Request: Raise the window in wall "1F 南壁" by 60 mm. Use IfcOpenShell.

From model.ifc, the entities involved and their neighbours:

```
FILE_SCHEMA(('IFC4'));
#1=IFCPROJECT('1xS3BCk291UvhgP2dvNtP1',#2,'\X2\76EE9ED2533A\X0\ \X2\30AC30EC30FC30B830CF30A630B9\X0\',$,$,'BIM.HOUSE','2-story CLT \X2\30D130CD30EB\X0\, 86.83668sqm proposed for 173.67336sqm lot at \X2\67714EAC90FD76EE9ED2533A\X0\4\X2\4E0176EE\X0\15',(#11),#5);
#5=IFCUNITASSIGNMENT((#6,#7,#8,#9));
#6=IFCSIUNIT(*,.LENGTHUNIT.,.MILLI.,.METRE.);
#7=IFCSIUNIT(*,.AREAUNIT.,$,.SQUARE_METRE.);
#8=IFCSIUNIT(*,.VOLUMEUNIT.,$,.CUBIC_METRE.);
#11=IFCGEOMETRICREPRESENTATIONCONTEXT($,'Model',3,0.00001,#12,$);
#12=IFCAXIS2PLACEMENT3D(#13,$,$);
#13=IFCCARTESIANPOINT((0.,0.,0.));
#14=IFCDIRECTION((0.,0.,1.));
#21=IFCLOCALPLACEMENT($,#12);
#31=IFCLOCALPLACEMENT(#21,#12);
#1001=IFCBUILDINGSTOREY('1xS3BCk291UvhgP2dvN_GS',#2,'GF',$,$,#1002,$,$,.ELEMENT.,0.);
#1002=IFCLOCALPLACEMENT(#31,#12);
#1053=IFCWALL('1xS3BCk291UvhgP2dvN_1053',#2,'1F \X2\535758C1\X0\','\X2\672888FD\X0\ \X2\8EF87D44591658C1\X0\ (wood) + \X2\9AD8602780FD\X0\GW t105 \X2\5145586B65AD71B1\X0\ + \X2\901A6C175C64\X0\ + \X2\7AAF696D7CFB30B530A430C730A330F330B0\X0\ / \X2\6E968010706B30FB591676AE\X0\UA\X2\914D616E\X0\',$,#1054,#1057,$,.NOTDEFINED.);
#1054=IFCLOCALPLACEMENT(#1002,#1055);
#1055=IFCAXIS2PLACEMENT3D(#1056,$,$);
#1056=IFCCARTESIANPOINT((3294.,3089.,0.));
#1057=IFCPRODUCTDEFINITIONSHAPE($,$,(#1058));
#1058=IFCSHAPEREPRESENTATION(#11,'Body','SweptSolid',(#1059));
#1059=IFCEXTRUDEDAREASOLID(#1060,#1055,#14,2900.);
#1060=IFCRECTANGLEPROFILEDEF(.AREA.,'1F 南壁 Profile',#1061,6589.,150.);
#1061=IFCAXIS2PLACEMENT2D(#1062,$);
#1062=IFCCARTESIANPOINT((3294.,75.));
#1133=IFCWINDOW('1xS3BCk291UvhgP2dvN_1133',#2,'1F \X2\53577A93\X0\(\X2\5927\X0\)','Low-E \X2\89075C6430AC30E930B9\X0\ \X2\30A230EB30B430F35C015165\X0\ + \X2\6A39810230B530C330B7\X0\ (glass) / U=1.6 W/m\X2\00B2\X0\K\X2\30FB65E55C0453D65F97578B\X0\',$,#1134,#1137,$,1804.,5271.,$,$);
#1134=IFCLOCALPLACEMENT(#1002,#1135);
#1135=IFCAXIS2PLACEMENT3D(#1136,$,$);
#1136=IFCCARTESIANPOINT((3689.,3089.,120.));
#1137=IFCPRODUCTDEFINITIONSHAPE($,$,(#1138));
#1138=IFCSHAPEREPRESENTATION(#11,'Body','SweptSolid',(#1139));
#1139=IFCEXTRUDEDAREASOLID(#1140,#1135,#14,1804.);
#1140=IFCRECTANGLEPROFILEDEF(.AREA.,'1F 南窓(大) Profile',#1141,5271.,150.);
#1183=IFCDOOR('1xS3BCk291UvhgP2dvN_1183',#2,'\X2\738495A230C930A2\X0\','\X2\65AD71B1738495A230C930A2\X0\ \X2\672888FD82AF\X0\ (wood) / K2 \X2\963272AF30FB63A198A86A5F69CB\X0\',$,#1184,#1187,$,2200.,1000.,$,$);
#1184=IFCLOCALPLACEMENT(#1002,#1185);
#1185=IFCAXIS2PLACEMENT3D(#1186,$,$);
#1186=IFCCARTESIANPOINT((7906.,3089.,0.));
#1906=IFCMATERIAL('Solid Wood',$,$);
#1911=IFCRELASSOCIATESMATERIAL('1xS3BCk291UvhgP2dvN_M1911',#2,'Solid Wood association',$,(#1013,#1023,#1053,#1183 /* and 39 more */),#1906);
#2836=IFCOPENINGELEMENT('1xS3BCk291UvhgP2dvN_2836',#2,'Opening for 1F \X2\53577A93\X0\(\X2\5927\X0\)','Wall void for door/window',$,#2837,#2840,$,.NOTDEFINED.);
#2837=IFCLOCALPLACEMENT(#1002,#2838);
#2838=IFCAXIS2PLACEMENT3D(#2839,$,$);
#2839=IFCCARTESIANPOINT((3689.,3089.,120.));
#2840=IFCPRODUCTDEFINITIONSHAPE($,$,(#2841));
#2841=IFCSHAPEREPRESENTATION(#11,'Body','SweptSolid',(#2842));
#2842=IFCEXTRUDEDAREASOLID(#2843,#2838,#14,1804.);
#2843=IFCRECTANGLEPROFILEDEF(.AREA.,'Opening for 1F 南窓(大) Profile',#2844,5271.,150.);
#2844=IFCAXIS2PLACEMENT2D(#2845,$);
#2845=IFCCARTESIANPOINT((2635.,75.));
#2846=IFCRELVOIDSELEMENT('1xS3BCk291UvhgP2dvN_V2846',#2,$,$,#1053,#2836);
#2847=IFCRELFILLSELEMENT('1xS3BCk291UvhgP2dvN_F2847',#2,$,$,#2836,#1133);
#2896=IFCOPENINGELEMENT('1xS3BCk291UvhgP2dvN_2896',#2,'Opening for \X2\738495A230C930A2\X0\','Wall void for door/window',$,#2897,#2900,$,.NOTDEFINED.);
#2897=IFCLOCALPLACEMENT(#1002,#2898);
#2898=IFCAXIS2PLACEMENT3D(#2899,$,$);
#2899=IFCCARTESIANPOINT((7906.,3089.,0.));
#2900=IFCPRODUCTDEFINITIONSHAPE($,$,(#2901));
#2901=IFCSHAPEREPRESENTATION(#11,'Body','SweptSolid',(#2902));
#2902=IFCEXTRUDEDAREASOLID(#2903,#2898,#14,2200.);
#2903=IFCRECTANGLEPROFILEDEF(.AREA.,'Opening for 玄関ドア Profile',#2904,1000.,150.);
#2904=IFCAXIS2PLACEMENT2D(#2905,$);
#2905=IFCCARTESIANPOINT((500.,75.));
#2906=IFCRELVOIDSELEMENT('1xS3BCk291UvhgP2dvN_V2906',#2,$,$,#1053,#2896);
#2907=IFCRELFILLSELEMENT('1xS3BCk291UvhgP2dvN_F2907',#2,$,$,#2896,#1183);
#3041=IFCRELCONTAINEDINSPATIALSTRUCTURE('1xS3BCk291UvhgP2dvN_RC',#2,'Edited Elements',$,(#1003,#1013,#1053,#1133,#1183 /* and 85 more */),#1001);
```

```python
import numpy as np
import ifcopenshell
import ifcopenshell.api.geometry
import ifcopenshell.util.placement
import ifcopenshell.util.unit

model = ifcopenshell.open("model.ifc")
unit_scale = ifcopenshell.util.unit.calculate_unit_scale(model)

window = model.by_guid("1xS3BCk291UvhgP2dvN_1133")
opening = window.FillsVoids[0].RelatingOpeningElement
dz = 0.06 / unit_scale

shift = np.array([0.0, 0.0, dz])
# The window is not placed relative to its opening, so move both.
for product in (opening, window):
    matrix = ifcopenshell.util.placement.get_local_placement(product.ObjectPlacement)
    matrix[:3, 3] += shift
    ifcopenshell.api.geometry.edit_object_placement(model, product=product, matrix=matrix, is_si=False)

print(f"moved by {dz * unit_scale:+.3f} m")

model.write("model-out.ifc")
```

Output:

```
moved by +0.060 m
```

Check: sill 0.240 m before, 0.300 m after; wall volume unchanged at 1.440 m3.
